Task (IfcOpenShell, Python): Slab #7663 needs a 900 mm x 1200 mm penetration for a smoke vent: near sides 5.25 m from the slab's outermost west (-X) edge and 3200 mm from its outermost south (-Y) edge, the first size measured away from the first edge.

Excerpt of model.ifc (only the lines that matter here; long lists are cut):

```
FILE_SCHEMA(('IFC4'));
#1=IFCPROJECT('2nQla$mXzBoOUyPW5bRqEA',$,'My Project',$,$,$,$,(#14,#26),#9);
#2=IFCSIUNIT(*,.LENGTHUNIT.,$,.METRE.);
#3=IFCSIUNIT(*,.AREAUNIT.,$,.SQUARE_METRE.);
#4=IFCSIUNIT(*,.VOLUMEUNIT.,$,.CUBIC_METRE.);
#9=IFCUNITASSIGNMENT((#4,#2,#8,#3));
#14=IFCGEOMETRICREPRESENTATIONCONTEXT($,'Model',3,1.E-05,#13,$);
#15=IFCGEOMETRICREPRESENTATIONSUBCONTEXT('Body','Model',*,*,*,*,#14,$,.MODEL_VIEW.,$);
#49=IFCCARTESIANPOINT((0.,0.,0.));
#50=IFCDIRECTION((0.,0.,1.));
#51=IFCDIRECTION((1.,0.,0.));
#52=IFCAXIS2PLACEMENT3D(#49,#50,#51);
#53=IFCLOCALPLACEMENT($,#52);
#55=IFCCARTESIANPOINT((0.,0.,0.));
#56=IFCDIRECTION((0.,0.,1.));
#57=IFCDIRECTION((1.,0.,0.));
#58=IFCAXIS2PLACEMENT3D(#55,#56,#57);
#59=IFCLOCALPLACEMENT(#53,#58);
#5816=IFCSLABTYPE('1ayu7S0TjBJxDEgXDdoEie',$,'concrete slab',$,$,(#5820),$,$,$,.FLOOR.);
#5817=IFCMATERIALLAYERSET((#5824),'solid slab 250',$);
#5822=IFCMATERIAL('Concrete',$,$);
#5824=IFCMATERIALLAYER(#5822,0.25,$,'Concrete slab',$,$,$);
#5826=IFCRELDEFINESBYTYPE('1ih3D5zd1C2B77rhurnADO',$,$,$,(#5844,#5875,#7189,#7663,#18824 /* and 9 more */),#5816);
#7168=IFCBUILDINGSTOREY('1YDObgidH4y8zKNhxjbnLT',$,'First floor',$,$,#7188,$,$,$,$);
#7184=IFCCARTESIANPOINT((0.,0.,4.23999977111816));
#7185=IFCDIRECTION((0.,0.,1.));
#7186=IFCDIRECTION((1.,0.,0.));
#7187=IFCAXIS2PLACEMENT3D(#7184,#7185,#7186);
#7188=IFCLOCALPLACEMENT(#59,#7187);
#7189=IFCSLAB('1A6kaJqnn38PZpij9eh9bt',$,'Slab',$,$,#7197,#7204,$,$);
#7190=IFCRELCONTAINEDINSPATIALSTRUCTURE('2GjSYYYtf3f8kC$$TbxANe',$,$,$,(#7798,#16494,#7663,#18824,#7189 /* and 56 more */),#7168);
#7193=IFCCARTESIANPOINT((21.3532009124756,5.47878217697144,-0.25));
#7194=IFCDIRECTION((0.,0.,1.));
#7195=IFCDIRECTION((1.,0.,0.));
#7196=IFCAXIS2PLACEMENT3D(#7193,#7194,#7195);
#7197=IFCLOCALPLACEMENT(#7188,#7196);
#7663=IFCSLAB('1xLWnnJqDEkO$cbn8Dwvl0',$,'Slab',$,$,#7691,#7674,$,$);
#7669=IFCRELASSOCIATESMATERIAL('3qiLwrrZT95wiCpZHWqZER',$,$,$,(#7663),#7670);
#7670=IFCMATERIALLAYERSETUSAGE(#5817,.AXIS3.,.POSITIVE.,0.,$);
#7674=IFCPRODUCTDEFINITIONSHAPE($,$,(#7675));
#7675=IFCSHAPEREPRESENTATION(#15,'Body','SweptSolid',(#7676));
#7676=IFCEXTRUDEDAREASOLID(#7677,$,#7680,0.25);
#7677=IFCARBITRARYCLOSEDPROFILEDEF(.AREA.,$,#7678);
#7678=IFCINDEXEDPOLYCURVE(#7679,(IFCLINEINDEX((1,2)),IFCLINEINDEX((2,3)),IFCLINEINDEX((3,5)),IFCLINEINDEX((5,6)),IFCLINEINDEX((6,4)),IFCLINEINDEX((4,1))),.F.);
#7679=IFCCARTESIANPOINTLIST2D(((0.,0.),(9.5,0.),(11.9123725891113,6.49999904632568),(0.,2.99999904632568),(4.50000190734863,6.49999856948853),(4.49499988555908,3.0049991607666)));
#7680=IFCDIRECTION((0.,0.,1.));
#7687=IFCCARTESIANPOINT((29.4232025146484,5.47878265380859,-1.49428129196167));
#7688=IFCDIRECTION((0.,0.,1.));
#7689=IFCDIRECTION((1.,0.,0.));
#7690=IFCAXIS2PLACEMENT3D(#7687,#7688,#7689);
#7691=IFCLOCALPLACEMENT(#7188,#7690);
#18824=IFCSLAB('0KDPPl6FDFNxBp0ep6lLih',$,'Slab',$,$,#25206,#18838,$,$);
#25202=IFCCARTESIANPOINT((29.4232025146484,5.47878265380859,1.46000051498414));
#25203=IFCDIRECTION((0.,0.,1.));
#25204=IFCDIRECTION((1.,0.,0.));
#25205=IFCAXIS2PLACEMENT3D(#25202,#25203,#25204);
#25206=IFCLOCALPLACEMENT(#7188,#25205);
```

```python
import numpy as np
import ifcopenshell
import ifcopenshell.api.feature
import ifcopenshell.api.geometry
import ifcopenshell.api.root
import ifcopenshell.geom
import ifcopenshell.util.placement
import ifcopenshell.util.representation
import ifcopenshell.util.shape
import ifcopenshell.util.unit

model = ifcopenshell.open("model.ifc")
unit_scale = ifcopenshell.util.unit.calculate_unit_scale(model)
settings = ifcopenshell.geom.settings()


def volume(element):
    """Net volume in cubic metres, openings subtracted."""
    shape = ifcopenshell.geom.create_shape(settings, element)
    return ifcopenshell.util.shape.get_volume(shape.geometry)


slab = model.by_guid("1xLWnnJqDEkO$cbn8Dwvl0")
before = volume(slab)

# Extent in the slab's own axes, in metres. The edges named are its -X and -Y sides.
slab_shape = ifcopenshell.geom.create_shape(settings, slab)
vertices = ifcopenshell.util.shape.get_vertices(slab_shape.geometry)
x_min, y_min, bottom = vertices.min(axis=0)
top = vertices[:, 2].max()

opening = ifcopenshell.api.root.create_entity(model, ifc_class="IfcOpeningElement", name="Smoke vent opening", predefined_type="OPENING")
context = ifcopenshell.util.representation.get_context(model, "Model", "Body", "MODEL_VIEW")
width, depth = 0.9, 1.2
outline = [(0.0, 0.0), (width, 0.0), (width, depth), (0.0, depth), (0.0, 0.0)]
# Overshoot both faces by 50 mm so the cut is clean.
shape = ifcopenshell.api.geometry.add_slab_representation(
    model, context=context, depth=top - bottom + 0.1, polyline=outline
)
ifcopenshell.api.geometry.assign_representation(model, product=opening, representation=shape)

matrix = ifcopenshell.util.placement.get_local_placement(slab.ObjectPlacement)
matrix[:, 3] = matrix @ np.append(np.array([x_min + 5.25, y_min + 3.2, bottom - 0.05]) / unit_scale, 1.0)
ifcopenshell.api.geometry.edit_object_placement(model, product=opening, matrix=matrix, is_si=False)
ifcopenshell.api.feature.add_feature(model, feature=opening, element=slab)

after = volume(slab)

print(f"slab volume {before:.3f} -> {after:.3f} m3")

model.write("model_rev.ifc")
```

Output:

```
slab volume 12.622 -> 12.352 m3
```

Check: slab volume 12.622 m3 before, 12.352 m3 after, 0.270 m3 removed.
